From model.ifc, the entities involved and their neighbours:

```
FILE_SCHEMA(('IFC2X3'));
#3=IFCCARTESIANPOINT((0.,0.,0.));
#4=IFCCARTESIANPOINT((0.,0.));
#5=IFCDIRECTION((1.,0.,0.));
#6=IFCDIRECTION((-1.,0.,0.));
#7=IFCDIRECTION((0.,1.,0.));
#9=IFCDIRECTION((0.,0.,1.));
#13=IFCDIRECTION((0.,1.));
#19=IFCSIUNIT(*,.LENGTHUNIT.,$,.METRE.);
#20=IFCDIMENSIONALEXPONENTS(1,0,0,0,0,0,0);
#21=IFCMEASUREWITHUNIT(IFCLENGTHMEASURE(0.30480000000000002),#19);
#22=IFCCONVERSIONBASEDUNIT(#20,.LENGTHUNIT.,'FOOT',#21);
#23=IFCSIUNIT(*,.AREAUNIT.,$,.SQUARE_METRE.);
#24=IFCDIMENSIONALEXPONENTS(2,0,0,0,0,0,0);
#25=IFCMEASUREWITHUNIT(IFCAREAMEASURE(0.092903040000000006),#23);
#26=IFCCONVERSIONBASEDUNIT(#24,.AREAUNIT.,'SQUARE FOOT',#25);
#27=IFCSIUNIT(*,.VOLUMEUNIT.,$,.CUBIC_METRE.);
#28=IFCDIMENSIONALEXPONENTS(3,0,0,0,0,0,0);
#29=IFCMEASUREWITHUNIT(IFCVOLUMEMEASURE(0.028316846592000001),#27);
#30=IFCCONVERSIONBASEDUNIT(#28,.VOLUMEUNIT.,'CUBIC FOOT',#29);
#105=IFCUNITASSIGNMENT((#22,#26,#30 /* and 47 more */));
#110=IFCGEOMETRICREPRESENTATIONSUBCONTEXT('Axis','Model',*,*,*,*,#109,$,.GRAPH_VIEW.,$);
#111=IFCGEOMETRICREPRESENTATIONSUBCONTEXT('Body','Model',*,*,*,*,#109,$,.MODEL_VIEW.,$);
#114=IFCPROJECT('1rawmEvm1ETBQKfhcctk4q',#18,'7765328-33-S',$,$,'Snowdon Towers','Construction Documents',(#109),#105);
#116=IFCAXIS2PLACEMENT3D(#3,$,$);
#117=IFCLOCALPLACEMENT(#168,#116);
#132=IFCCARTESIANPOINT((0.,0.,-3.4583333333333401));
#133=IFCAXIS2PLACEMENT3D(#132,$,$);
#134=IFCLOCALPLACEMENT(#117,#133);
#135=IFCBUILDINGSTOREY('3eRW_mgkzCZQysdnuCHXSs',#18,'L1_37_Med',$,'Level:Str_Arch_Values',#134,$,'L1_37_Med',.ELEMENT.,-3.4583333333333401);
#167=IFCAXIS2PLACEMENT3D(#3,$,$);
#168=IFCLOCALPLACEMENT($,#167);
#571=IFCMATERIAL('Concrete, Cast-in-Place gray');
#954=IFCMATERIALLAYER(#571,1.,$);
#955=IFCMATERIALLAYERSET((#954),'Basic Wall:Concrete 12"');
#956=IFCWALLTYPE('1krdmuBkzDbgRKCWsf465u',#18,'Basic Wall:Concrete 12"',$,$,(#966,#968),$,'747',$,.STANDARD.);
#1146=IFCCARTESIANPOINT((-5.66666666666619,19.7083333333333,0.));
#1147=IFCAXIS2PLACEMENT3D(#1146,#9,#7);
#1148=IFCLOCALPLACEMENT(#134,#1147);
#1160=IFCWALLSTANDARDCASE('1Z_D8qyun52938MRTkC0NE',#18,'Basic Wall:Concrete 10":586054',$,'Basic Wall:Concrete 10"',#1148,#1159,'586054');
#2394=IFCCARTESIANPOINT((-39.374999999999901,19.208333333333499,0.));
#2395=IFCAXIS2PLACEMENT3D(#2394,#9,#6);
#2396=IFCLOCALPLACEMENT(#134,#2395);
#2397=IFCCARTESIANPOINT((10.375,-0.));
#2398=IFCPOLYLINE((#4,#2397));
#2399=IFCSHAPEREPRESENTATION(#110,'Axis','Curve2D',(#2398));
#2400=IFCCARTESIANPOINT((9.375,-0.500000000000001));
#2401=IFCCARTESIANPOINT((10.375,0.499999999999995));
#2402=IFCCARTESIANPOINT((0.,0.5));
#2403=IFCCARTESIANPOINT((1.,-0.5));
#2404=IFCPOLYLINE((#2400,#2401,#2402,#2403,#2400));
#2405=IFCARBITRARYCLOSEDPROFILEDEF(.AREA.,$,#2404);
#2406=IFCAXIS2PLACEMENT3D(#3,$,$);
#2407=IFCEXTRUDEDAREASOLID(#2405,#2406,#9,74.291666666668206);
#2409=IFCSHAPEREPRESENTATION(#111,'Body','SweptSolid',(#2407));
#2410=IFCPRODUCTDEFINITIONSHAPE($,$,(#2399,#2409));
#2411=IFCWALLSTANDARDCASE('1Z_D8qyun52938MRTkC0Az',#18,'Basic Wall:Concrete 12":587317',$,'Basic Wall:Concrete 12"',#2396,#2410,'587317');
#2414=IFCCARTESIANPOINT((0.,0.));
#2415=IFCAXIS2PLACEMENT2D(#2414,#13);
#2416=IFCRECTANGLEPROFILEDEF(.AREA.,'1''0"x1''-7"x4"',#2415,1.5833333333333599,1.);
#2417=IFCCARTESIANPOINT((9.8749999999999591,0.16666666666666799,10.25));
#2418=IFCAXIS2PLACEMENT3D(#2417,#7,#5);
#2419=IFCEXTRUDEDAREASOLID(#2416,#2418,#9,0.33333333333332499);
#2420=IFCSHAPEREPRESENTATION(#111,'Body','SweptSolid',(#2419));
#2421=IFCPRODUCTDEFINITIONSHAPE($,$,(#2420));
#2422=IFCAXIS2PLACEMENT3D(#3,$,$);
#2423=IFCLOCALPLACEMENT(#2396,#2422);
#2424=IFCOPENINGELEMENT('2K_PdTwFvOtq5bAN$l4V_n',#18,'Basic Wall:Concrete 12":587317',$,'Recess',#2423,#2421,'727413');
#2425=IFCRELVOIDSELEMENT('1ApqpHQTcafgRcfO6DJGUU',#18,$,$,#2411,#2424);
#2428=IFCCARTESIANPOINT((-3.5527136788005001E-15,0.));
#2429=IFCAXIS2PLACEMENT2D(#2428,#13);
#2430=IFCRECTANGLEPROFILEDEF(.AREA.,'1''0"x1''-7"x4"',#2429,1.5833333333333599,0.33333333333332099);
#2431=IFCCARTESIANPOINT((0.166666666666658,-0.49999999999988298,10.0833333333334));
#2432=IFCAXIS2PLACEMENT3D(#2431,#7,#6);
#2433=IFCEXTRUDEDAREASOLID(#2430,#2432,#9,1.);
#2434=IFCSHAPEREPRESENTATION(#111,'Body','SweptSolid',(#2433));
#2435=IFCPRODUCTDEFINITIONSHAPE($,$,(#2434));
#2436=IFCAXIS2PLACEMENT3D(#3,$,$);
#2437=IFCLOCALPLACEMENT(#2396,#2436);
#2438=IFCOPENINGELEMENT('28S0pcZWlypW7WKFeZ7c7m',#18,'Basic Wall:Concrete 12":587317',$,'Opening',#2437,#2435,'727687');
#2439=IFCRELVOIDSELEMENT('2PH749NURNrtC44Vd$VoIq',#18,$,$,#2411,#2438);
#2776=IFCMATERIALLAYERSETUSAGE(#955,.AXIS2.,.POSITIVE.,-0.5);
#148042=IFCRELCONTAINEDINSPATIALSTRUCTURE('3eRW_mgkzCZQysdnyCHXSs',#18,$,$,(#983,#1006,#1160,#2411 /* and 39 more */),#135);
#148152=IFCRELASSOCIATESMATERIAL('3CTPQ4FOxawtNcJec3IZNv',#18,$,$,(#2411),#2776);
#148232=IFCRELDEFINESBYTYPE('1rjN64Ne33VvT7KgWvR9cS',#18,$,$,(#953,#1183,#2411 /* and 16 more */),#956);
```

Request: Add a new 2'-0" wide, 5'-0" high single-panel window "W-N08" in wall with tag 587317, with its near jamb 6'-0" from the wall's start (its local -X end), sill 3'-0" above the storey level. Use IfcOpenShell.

```python
import numpy as np
import ifcopenshell
import ifcopenshell.api.feature
import ifcopenshell.api.geometry
import ifcopenshell.api.root
import ifcopenshell.api.spatial
import ifcopenshell.api.type
import ifcopenshell.geom
import ifcopenshell.util.element
import ifcopenshell.util.placement
import ifcopenshell.util.representation
import ifcopenshell.util.shape
import ifcopenshell.util.unit

model = ifcopenshell.open("model.ifc")
unit_scale = ifcopenshell.util.unit.calculate_unit_scale(model)
settings = ifcopenshell.geom.settings()


def volume(element):
    """Net volume in cubic metres, openings subtracted."""
    shape = ifcopenshell.geom.create_shape(settings, element)
    return ifcopenshell.util.shape.get_volume(shape.geometry)


wall = model.by_guid("1Z_D8qyun52938MRTkC0Az")
storey = ifcopenshell.util.element.get_container(wall, ifc_class="IfcBuildingStorey")
context = ifcopenshell.util.representation.get_context(model, "Model", "Body", "MODEL_VIEW")
before = volume(wall)

width, height, from_end, sill = 0.6096, 1.524, 1.8288, 0.9144  # metres

# The wall runs along its own X axis, and the end named is its -X end.
wall_shape = ifcopenshell.geom.create_shape(settings, wall)
x, y, z = ifcopenshell.util.shape.get_vertices(wall_shape.geometry).T
start = x.min() + from_end
face, thickness = float(y.min()), float(y.max() - y.min())
wall_matrix = ifcopenshell.util.placement.get_local_placement(wall.ObjectPlacement)
level = ifcopenshell.util.placement.get_local_placement(storey.ObjectPlacement)[2, 3]


def in_wall(x, y):
    """Placement at x, y metres in the wall's axes, at sill height."""
    matrix = wall_matrix.copy()
    matrix[:, 3] = wall_matrix @ np.array([x / unit_scale, y / unit_scale, 0.0, 1.0])
    matrix[2, 3] = level + sill / unit_scale
    return matrix


# Opening: a box that overshoots both wall faces by 50 mm.
opening = ifcopenshell.api.root.create_entity(model, ifc_class="IfcOpeningElement")
box = ifcopenshell.api.geometry.add_wall_representation(
    model, context=context, length=width, height=height, thickness=thickness + 0.1
)
ifcopenshell.api.geometry.assign_representation(model, product=opening, representation=box)
ifcopenshell.api.geometry.edit_object_placement(model, product=opening, matrix=in_wall(start, face - 0.05), is_si=False)
ifcopenshell.api.feature.add_feature(model, feature=opening, element=wall)

window = ifcopenshell.api.root.create_entity(model, ifc_class="IfcWindow", name="W-N08")
window.OverallWidth, window.OverallHeight = width / unit_scale, height / unit_scale
body = ifcopenshell.api.geometry.add_window_representation(
    model,
    context=context,
    overall_width=window.OverallWidth,
    overall_height=window.OverallHeight,
    partition_type="SINGLE_PANEL",
)
ifcopenshell.api.geometry.assign_representation(model, product=window, representation=body)
ifcopenshell.api.spatial.assign_container(model, products=[window], relating_structure=storey)
fills = ifcopenshell.api.feature.add_filling(model, opening=opening, element=window)
fills.OwnerHistory = window.OwnerHistory  # required in IFC2X3

# IFC2X3 keeps the operation on the window style.
style = ifcopenshell.api.root.create_entity(model, ifc_class="IfcWindowStyle", name="W-N08")
style.OperationType, style.ConstructionType = "SINGLE_PANEL", "NOTDEFINED"
style.ParameterTakesPrecedence = style.Sizeable = False
ifcopenshell.api.type.assign_type(model, related_objects=[window], relating_type=style)

# Centre the window in the wall's thickness.
ifcopenshell.api.geometry.edit_object_placement(model, product=window, matrix=in_wall(start, face), is_si=False)
window_shape = ifcopenshell.geom.create_shape(settings, window)
depth = ifcopenshell.util.shape.get_vertices(window_shape.geometry)[:, 1]
offset = face + thickness / 2 - (depth.min() + depth.max()) / 2
ifcopenshell.api.geometry.edit_object_placement(model, product=window, matrix=in_wall(start, offset), is_si=False)

after = volume(wall)

print(f"wall volume {before:.3f} -> {after:.3f} m3")

model.write("model_updated.ifc")
```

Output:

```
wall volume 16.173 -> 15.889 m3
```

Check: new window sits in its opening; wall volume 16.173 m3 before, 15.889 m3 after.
